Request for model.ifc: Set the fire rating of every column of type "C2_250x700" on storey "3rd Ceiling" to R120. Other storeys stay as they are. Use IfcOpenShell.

First a look at what the model holds.

```python
import ifcopenshell
import ifcopenshell.util.element

model = ifcopenshell.open("model.ifc")
print(model.schema)
storey = next(s for s in model.by_type("IfcBuildingStorey") if s.Name == "3rd Ceiling")
columns = [e for e in ifcopenshell.util.element.get_decomposition(storey) if e.is_a("IfcColumn")]
seen = {}
for e in columns:
    element_type = ifcopenshell.util.element.get_type(e)
    key = (element_type.Name if element_type != e and element_type else None, ifcopenshell.util.element.get_pset(e, "Pset_ColumnCommon", "FireRating"))
    seen[key] = seen.get(key, 0) + 1
for (name, value), count in sorted(seen.items(), key=str):
    print(count, "x", name, "|", value)
```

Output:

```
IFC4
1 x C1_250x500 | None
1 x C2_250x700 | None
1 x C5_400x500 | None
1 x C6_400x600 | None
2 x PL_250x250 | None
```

```python
import ifcopenshell
import ifcopenshell.api.pset
import ifcopenshell.util.element

model = ifcopenshell.open("model.ifc")

storey = next(s for s in model.by_type("IfcBuildingStorey") if s.Name == "3rd Ceiling")
columns = [e for e in ifcopenshell.util.element.get_decomposition(storey) if e.is_a("IfcColumn")]

count = 0
for e in columns:
    element_type = ifcopenshell.util.element.get_type(e)
    if element_type in (None, e) or element_type.Name != "C2_250x700":
        continue
    # add_pset returns the element's existing set when there is one.
    pset = ifcopenshell.api.pset.add_pset(model, product=e, name="Pset_ColumnCommon")
    ifcopenshell.api.pset.edit_pset(model, pset=pset, properties={"FireRating": "R120"})
    count += 1

print(count, "columns updated")

model.write("model_edited.ifc")
```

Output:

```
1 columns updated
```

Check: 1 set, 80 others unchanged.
